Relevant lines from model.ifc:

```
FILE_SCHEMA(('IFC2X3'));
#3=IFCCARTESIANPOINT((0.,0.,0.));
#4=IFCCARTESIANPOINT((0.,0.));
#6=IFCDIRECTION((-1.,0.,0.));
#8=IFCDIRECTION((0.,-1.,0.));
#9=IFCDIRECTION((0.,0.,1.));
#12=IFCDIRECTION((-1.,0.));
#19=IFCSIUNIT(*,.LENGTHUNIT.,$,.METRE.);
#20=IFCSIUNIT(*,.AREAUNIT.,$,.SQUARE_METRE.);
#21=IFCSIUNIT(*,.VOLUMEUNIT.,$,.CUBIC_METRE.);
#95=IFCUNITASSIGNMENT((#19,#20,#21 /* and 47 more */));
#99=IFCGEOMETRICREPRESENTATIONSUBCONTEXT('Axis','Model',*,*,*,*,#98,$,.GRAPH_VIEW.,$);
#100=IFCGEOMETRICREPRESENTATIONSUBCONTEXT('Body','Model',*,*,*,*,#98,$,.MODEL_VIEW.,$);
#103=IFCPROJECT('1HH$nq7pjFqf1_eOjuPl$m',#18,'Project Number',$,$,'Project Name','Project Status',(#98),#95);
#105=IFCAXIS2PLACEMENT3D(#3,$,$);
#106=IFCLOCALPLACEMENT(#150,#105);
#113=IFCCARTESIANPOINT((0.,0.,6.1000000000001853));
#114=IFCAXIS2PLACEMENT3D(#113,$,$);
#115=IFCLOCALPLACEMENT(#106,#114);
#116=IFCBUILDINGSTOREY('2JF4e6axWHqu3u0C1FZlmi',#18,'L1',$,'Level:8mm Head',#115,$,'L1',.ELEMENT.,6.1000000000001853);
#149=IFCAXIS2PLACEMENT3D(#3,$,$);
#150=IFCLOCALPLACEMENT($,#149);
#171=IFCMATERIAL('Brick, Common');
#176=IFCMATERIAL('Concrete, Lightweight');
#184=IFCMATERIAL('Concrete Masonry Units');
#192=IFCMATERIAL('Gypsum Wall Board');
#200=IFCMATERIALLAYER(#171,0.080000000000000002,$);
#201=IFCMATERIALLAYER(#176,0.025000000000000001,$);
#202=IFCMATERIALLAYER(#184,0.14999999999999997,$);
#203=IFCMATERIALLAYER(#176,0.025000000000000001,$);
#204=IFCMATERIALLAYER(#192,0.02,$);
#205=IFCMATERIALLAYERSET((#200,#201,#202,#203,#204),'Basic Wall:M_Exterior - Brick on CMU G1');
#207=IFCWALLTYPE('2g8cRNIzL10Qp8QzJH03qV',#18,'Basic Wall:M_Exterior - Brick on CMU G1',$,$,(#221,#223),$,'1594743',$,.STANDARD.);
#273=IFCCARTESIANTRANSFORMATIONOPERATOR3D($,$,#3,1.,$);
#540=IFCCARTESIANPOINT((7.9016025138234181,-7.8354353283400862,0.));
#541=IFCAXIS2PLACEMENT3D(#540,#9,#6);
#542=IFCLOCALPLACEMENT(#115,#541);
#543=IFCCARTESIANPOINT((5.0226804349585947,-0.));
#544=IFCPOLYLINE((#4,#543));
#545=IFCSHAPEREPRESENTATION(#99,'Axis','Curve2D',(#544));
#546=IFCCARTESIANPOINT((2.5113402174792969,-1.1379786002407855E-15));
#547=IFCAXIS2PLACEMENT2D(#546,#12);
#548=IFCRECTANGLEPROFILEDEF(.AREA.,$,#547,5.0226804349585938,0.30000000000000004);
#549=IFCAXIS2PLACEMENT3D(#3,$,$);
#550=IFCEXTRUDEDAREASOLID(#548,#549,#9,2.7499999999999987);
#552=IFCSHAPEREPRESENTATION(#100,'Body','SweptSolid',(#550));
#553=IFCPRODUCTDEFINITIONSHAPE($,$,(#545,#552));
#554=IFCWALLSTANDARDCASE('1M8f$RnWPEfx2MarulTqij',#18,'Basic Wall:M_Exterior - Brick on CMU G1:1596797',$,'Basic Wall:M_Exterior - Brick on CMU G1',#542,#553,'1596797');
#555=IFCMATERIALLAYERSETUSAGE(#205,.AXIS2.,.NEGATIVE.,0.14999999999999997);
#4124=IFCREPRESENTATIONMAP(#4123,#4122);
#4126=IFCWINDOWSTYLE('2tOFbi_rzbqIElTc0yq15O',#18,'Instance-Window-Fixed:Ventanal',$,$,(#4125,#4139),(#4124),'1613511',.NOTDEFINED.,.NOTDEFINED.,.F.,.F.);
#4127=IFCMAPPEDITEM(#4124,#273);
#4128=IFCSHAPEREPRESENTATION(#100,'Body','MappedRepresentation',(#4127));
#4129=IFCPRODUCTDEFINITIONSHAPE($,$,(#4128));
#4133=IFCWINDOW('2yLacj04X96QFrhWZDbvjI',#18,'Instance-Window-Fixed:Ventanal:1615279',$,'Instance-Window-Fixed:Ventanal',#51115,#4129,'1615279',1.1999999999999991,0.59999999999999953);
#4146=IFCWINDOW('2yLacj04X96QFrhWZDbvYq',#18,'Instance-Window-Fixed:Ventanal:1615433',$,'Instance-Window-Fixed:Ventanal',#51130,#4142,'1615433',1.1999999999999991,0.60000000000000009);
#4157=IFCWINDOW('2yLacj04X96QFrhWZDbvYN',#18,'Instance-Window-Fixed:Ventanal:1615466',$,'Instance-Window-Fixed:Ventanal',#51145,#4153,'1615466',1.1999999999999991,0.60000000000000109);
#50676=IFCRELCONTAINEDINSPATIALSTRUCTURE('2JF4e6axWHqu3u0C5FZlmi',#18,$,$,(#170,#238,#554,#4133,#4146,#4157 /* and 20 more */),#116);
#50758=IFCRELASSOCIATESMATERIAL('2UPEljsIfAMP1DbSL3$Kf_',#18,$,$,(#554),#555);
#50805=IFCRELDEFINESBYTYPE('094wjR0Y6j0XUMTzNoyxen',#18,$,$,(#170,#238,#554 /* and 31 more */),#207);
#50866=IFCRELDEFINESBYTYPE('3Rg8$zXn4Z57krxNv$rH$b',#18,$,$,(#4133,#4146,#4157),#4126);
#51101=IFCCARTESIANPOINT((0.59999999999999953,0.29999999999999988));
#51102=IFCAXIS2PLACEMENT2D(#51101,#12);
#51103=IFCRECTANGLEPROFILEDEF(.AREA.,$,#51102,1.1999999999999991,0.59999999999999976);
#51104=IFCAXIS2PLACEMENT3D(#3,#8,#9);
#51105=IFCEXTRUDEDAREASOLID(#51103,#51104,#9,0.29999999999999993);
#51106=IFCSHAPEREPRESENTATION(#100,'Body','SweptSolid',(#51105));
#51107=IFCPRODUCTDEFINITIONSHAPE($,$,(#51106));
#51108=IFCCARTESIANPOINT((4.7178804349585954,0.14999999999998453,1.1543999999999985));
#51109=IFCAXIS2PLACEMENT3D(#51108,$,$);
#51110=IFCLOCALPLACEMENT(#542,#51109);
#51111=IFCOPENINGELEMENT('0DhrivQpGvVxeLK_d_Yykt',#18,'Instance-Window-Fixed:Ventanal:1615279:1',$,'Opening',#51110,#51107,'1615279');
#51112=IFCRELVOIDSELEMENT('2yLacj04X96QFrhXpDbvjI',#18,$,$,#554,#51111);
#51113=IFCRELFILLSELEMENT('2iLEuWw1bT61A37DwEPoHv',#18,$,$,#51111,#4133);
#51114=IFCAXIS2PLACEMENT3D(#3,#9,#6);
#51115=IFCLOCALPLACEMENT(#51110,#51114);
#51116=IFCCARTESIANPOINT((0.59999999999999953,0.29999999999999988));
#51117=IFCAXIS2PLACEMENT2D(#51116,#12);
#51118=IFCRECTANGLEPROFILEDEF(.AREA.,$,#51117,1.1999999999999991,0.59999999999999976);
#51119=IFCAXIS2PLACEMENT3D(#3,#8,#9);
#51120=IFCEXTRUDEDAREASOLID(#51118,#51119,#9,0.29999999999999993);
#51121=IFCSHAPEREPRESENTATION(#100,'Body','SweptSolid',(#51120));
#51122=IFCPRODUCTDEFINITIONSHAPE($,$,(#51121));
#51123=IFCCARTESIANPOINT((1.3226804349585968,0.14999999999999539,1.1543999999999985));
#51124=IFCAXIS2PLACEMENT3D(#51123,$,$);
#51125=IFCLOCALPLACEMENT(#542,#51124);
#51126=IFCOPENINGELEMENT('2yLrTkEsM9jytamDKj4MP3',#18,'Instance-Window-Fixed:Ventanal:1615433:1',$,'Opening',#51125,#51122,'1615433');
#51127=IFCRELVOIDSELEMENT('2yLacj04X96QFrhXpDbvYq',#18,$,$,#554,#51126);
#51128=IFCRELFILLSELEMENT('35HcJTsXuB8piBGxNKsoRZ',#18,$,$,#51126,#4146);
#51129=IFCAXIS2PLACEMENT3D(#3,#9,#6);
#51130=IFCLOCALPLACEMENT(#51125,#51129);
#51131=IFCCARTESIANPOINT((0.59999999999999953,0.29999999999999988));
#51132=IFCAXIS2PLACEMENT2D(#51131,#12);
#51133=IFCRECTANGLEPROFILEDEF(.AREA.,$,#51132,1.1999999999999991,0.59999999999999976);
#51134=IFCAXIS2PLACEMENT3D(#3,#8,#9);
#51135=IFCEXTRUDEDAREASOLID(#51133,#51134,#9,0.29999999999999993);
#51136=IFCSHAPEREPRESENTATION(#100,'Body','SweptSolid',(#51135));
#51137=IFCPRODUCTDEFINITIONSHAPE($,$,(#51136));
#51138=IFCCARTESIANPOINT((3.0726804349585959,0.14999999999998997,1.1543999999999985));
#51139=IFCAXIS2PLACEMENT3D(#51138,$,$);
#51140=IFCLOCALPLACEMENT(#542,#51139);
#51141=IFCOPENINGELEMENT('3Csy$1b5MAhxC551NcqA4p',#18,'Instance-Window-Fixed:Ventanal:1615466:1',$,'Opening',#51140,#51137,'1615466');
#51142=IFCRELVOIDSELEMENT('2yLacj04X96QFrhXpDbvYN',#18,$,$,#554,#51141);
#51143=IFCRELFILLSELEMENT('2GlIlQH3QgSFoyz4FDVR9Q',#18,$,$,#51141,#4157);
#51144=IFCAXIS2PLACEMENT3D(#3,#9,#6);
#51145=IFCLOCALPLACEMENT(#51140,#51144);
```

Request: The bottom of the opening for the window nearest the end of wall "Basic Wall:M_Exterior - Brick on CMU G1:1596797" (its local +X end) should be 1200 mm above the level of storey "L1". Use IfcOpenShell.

```python
import numpy as np
import ifcopenshell
import ifcopenshell.api.geometry
import ifcopenshell.geom
import ifcopenshell.util.element
import ifcopenshell.util.placement
import ifcopenshell.util.shape
import ifcopenshell.util.unit

model = ifcopenshell.open("model.ifc")
unit_scale = ifcopenshell.util.unit.calculate_unit_scale(model)

window = model.by_guid("2yLacj04X96QFrhWZDbvjI")
opening = window.FillsVoids[0].RelatingOpeningElement
storey = ifcopenshell.util.element.get_container(window, ifc_class="IfcBuildingStorey")
level = ifcopenshell.util.placement.get_local_placement(storey.ObjectPlacement)[2, 3]

# The opening's origin need not be at the sill, so measure its lowest point.
shape = ifcopenshell.geom.create_shape(ifcopenshell.geom.settings(), opening)
bottom = ifcopenshell.util.shape.get_shape_bottom_elevation(shape, shape.geometry) / unit_scale
dz = level + 1.2 / unit_scale - bottom

shift = np.array([0.0, 0.0, dz])
# The window is placed relative to its opening, so it follows when the opening moves.
matrix = ifcopenshell.util.placement.get_local_placement(opening.ObjectPlacement)
matrix[:3, 3] += shift
ifcopenshell.api.geometry.edit_object_placement(
    model, product=opening, matrix=matrix, is_si=False, should_transform_children=True
)

print(f"moved by {dz * unit_scale:+.3f} m")

model.write("model_rev.ifc")
```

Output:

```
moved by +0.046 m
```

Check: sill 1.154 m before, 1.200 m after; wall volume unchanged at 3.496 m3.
